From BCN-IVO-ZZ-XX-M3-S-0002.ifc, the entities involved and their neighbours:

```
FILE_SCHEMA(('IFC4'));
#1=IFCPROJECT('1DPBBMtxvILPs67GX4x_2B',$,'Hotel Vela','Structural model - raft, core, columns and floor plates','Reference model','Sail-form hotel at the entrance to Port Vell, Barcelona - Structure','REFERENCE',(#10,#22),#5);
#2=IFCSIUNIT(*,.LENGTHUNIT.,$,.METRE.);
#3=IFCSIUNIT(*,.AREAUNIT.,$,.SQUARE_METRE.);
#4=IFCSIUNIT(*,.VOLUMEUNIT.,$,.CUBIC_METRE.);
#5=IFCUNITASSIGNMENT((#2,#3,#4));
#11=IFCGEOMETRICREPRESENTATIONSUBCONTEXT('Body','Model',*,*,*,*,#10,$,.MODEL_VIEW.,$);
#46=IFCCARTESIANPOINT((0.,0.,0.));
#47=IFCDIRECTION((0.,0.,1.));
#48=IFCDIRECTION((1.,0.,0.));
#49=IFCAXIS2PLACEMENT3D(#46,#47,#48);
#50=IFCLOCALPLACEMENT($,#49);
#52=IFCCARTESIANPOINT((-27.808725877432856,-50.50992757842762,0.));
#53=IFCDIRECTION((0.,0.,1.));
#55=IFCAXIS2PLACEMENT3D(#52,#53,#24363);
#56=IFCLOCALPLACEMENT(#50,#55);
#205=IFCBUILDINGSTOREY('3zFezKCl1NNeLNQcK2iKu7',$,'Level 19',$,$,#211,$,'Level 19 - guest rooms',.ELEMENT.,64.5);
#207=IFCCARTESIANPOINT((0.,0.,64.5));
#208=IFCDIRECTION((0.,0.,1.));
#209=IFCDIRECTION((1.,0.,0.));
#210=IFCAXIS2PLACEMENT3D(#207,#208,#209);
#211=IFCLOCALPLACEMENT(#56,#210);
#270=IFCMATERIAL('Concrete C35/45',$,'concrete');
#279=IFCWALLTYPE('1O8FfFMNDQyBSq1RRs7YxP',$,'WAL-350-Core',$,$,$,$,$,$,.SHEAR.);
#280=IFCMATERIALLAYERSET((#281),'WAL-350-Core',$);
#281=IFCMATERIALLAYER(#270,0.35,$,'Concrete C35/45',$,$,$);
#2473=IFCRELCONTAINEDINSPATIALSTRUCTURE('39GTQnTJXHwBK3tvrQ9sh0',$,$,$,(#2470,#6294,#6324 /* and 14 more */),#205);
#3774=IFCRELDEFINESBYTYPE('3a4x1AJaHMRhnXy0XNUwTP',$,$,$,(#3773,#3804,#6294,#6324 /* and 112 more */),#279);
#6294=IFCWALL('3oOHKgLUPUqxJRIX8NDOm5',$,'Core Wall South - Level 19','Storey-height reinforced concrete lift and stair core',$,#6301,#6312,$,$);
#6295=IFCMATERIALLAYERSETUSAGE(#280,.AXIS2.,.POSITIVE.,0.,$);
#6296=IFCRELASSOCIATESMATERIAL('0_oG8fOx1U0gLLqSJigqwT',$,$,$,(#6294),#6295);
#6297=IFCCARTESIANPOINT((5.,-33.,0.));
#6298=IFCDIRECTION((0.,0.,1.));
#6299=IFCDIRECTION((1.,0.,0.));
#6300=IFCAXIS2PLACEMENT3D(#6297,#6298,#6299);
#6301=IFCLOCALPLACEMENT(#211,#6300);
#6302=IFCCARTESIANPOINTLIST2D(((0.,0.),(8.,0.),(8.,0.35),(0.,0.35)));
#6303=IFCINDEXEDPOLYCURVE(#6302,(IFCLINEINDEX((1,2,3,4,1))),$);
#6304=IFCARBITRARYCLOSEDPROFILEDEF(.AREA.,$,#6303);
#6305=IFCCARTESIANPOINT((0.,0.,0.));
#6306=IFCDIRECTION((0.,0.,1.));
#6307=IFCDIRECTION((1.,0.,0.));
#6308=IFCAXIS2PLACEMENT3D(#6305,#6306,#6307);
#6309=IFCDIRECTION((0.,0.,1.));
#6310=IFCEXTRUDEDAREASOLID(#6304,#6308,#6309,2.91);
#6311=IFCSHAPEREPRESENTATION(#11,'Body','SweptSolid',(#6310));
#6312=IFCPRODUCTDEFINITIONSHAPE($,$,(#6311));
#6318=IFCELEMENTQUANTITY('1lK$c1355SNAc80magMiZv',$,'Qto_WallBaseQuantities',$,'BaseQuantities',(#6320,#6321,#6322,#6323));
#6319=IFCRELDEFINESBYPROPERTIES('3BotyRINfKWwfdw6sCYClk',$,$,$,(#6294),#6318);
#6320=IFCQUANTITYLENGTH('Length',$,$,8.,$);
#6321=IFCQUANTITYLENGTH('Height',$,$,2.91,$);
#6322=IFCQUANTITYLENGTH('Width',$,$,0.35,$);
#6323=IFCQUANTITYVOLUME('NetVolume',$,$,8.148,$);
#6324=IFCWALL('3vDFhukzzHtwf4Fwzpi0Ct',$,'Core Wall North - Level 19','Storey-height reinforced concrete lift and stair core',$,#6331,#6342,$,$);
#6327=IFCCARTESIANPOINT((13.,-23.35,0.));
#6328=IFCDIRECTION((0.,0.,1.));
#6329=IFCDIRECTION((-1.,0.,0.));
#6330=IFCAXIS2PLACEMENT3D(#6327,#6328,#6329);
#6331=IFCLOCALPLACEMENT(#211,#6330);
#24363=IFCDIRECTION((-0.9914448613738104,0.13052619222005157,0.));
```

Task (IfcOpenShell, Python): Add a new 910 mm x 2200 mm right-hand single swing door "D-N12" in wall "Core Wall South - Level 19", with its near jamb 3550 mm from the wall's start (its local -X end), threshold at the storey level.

```python
import numpy as np
import ifcopenshell
import ifcopenshell.api.feature
import ifcopenshell.api.geometry
import ifcopenshell.api.pset
import ifcopenshell.api.root
import ifcopenshell.api.spatial
import ifcopenshell.geom
import ifcopenshell.util.element
import ifcopenshell.util.placement
import ifcopenshell.util.representation
import ifcopenshell.util.shape
import ifcopenshell.util.unit

model = ifcopenshell.open("BCN-IVO-ZZ-XX-M3-S-0002.ifc")
unit_scale = ifcopenshell.util.unit.calculate_unit_scale(model)
volume_scale = ifcopenshell.util.unit.calculate_unit_scale(model, "VOLUMEUNIT")
settings = ifcopenshell.geom.settings()


def volume(element):
    """Net volume in cubic metres, openings subtracted."""
    shape = ifcopenshell.geom.create_shape(settings, element)
    return ifcopenshell.util.shape.get_volume(shape.geometry)


wall = model.by_id(6294)
storey = ifcopenshell.util.element.get_container(wall, ifc_class="IfcBuildingStorey")
context = ifcopenshell.util.representation.get_context(model, "Model", "Body", "MODEL_VIEW")
before = volume(wall)

width, height, from_end, sill = 0.91, 2.2, 3.55, 0.0  # metres

# The wall runs along its own X axis, and the end named is its -X end.
wall_shape = ifcopenshell.geom.create_shape(settings, wall)
x, y, z = ifcopenshell.util.shape.get_vertices(wall_shape.geometry).T
start = x.min() + from_end
face, thickness = float(y.min()), float(y.max() - y.min())
wall_matrix = ifcopenshell.util.placement.get_local_placement(wall.ObjectPlacement)
level = ifcopenshell.util.placement.get_local_placement(storey.ObjectPlacement)[2, 3]


def in_wall(x, y):
    """Placement at x, y metres in the wall's axes, at sill height."""
    matrix = wall_matrix.copy()
    matrix[:, 3] = wall_matrix @ np.array([x / unit_scale, y / unit_scale, 0.0, 1.0])
    matrix[2, 3] = level + sill / unit_scale
    return matrix


# Opening: a box that overshoots both wall faces by 50 mm.
opening = ifcopenshell.api.root.create_entity(model, ifc_class="IfcOpeningElement", predefined_type="OPENING")
box = ifcopenshell.api.geometry.add_wall_representation(
    model, context=context, length=width, height=height, thickness=thickness + 0.1
)
ifcopenshell.api.geometry.assign_representation(model, product=opening, representation=box)
ifcopenshell.api.geometry.edit_object_placement(model, product=opening, matrix=in_wall(start, face - 0.05), is_si=False)
ifcopenshell.api.feature.add_feature(model, feature=opening, element=wall)

door = ifcopenshell.api.root.create_entity(model, ifc_class="IfcDoor", name="D-N12", predefined_type="DOOR")
door.OverallWidth, door.OverallHeight = width / unit_scale, height / unit_scale
door.OperationType = "SINGLE_SWING_RIGHT"
body = ifcopenshell.api.geometry.add_door_representation(
    model,
    context=context,
    overall_width=door.OverallWidth,
    overall_height=door.OverallHeight,
    operation_type="SINGLE_SWING_RIGHT",
    lining_properties={"LiningDepth": thickness / unit_scale, "ThresholdDepth": thickness / unit_scale},
)
ifcopenshell.api.geometry.assign_representation(model, product=door, representation=body)
ifcopenshell.api.spatial.assign_container(model, products=[door], relating_structure=storey)
ifcopenshell.api.feature.add_filling(model, opening=opening, element=door)

# The lining spans the wall, so the door starts at the wall face.
ifcopenshell.api.geometry.edit_object_placement(model, product=door, matrix=in_wall(start, face), is_si=False)

after = volume(wall)

# Update the wall's stored quantities.
qto = model.by_id(ifcopenshell.util.element.get_pset(wall, "Qto_WallBaseQuantities", should_inherit=False)["id"])
ifcopenshell.api.pset.edit_qto(model, qto=qto, properties={"NetVolume": after / volume_scale})

print(f"wall volume {before:.3f} -> {after:.3f} m3")

model.write("BCN-IVO-ZZ-XX-M3-S-0002-out.ifc")
```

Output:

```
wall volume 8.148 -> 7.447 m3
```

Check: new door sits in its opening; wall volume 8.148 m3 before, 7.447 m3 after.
